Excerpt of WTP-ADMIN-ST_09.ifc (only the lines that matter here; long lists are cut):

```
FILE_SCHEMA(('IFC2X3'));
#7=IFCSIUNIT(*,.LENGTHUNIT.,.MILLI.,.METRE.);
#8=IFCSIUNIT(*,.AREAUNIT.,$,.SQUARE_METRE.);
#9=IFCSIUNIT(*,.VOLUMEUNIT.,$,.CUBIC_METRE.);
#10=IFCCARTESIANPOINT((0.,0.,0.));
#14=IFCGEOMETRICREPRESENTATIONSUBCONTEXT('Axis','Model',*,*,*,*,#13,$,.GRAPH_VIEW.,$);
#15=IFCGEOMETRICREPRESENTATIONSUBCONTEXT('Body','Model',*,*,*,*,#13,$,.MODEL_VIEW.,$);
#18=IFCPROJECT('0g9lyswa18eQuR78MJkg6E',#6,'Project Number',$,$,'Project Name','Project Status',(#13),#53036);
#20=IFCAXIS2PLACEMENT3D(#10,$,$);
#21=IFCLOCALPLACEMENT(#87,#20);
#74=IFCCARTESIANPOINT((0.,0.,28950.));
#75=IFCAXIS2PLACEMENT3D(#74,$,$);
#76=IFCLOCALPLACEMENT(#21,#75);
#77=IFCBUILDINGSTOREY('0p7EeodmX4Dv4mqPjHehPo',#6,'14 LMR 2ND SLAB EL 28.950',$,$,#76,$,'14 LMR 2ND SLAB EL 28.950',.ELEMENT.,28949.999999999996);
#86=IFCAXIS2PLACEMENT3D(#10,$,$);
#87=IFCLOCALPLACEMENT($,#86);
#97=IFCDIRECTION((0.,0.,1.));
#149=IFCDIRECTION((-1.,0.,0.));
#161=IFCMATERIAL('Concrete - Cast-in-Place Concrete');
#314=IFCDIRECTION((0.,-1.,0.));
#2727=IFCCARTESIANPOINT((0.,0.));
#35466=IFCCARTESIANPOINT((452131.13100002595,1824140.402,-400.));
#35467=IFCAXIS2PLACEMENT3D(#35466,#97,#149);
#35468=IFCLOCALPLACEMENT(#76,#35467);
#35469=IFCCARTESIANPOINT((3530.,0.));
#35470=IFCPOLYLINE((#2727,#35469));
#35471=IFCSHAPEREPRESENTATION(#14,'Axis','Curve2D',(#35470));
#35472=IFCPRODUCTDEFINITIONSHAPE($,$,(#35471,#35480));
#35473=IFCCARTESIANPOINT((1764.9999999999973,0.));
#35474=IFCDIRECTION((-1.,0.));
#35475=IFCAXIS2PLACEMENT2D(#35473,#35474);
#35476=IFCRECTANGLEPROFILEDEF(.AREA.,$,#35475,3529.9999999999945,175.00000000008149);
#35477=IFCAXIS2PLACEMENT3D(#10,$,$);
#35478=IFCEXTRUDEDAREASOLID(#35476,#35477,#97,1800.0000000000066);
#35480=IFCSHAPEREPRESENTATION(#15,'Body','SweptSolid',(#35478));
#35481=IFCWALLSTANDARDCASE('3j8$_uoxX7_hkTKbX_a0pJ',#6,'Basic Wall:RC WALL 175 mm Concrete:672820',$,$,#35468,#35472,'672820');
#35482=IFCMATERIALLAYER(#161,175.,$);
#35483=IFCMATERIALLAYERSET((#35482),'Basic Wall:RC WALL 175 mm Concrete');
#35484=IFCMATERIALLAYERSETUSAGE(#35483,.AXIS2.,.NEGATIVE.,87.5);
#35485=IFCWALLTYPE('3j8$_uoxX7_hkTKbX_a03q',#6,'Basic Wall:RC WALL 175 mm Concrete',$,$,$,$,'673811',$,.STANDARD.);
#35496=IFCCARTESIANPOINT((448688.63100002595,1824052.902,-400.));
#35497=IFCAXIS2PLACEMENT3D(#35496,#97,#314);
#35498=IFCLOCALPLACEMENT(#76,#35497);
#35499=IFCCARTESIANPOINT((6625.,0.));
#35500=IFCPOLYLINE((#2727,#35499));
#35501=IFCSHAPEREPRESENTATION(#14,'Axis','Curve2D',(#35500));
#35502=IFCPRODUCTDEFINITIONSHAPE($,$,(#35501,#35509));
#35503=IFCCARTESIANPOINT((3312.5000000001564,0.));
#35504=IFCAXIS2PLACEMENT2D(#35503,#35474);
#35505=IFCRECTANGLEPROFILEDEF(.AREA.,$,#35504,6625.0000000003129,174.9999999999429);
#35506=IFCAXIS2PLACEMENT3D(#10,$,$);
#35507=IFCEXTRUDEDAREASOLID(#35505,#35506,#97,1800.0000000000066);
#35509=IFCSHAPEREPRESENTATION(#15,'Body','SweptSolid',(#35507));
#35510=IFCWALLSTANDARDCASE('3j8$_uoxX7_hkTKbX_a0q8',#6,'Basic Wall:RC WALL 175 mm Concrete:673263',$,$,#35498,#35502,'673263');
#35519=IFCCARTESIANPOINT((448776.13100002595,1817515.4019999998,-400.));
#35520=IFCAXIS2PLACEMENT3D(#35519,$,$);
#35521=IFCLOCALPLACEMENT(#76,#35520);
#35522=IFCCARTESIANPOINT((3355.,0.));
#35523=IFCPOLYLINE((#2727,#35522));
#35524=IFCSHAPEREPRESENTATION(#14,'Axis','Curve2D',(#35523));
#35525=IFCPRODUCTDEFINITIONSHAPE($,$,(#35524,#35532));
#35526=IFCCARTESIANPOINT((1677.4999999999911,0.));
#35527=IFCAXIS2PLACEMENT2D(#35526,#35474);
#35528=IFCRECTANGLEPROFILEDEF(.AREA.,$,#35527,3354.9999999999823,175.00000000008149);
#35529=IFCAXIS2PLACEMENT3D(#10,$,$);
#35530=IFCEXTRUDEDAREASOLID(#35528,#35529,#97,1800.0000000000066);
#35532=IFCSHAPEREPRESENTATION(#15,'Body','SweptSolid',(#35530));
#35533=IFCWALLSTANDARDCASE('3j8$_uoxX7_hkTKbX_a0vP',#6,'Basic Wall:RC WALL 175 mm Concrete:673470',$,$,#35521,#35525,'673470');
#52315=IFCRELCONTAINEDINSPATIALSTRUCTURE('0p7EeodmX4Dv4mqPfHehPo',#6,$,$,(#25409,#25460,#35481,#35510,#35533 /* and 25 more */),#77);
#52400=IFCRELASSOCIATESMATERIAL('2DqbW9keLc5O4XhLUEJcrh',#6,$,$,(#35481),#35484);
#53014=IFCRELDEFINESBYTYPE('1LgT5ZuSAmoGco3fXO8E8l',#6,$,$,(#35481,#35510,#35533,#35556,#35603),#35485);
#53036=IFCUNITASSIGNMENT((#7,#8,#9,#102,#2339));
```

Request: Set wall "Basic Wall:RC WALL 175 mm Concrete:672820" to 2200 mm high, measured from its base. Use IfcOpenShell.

```python
import ifcopenshell
import ifcopenshell.geom
import ifcopenshell.util.representation
import ifcopenshell.util.shape

model = ifcopenshell.open("WTP-ADMIN-ST_09.ifc")
settings = ifcopenshell.geom.settings()


def volume(element):
    """Net volume in cubic metres, openings subtracted."""
    shape = ifcopenshell.geom.create_shape(settings, element)
    return ifcopenshell.util.shape.get_volume(shape.geometry)


wall = model.by_guid("3j8$_uoxX7_hkTKbX_a0pJ")
before = volume(wall)

body = ifcopenshell.util.representation.get_representation(wall, "Model", "Body")
solid = body.Items[0]
old_height = solid.Depth
solid.Depth = 2200.0
after = volume(wall)

print(f"height {old_height:g} -> {solid.Depth:g}, volume {before:.3f} -> {after:.3f} m3")

model.write("WTP-ADMIN-ST_09_rev.ifc")
```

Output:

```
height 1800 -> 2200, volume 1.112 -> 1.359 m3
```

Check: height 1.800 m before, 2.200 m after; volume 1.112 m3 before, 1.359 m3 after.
